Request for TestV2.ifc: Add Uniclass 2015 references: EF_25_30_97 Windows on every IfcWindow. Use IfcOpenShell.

First a look at what the model holds.

```python
import ifcopenshell

model = ifcopenshell.open("TestV2.ifc")
print(model.schema)
print("classifications:", [c.Name for c in model.by_type("IfcClassification")])
for ifc_class in ("IfcDoor", "IfcRoof", "IfcStair", "IfcWall", "IfcWindow"):
    print(ifc_class, len(model.by_type(ifc_class)))
```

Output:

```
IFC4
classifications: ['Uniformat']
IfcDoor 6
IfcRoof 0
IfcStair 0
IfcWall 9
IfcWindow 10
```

```python
import ifcopenshell
import ifcopenshell.api.classification

model = ifcopenshell.open("TestV2.ifc")

system = ifcopenshell.api.classification.add_classification(model, classification="Uniclass 2015")

codes = {
    "IfcWindow": ("EF_25_30_97", "Windows"),
}
for ifc_class, (code, name) in codes.items():
    products = model.by_type(ifc_class)
    ifcopenshell.api.classification.add_reference(
        model, products=products, classification=system, identification=code, name=name
    )
    print(code, len(products))

model.write("TestV2_updated.ifc")
```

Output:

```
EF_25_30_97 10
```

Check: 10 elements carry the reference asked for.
